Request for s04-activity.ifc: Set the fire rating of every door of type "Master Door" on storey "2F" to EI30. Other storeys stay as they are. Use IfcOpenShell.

First a look at what the model holds.

```python
import ifcopenshell
import ifcopenshell.util.element

model = ifcopenshell.open("s04-activity.ifc")
print(model.schema)
storey = next(s for s in model.by_type("IfcBuildingStorey") if s.Name == "2F")
doors = [e for e in ifcopenshell.util.element.get_decomposition(storey) if e.is_a("IfcDoor")]
seen = {}
for e in doors:
    element_type = ifcopenshell.util.element.get_type(e)
    key = (element_type.Name if element_type != e and element_type else None, ifcopenshell.util.element.get_pset(e, "Pset_DoorCommon", "FireRating"))
    seen[key] = seen.get(key, 0) + 1
for (name, value), count in sorted(seen.items(), key=str):
    print(count, "x", name, "|", value)
```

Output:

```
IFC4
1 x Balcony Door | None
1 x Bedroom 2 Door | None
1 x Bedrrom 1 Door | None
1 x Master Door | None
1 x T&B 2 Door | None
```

```python
import ifcopenshell
import ifcopenshell.api.pset
import ifcopenshell.util.element

model = ifcopenshell.open("s04-activity.ifc")

storey = next(s for s in model.by_type("IfcBuildingStorey") if s.Name == "2F")
doors = [e for e in ifcopenshell.util.element.get_decomposition(storey) if e.is_a("IfcDoor")]

count = 0
for e in doors:
    element_type = ifcopenshell.util.element.get_type(e)
    if element_type in (None, e) or element_type.Name != "Master Door":
        continue
    # add_pset returns the element's existing set when there is one.
    pset = ifcopenshell.api.pset.add_pset(model, product=e, name="Pset_DoorCommon")
    ifcopenshell.api.pset.edit_pset(model, pset=pset, properties={"FireRating": "EI30"})
    count += 1

print(count, "doors updated")

model.write("s04-activity_v2.ifc")
```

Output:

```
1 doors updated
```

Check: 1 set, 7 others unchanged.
